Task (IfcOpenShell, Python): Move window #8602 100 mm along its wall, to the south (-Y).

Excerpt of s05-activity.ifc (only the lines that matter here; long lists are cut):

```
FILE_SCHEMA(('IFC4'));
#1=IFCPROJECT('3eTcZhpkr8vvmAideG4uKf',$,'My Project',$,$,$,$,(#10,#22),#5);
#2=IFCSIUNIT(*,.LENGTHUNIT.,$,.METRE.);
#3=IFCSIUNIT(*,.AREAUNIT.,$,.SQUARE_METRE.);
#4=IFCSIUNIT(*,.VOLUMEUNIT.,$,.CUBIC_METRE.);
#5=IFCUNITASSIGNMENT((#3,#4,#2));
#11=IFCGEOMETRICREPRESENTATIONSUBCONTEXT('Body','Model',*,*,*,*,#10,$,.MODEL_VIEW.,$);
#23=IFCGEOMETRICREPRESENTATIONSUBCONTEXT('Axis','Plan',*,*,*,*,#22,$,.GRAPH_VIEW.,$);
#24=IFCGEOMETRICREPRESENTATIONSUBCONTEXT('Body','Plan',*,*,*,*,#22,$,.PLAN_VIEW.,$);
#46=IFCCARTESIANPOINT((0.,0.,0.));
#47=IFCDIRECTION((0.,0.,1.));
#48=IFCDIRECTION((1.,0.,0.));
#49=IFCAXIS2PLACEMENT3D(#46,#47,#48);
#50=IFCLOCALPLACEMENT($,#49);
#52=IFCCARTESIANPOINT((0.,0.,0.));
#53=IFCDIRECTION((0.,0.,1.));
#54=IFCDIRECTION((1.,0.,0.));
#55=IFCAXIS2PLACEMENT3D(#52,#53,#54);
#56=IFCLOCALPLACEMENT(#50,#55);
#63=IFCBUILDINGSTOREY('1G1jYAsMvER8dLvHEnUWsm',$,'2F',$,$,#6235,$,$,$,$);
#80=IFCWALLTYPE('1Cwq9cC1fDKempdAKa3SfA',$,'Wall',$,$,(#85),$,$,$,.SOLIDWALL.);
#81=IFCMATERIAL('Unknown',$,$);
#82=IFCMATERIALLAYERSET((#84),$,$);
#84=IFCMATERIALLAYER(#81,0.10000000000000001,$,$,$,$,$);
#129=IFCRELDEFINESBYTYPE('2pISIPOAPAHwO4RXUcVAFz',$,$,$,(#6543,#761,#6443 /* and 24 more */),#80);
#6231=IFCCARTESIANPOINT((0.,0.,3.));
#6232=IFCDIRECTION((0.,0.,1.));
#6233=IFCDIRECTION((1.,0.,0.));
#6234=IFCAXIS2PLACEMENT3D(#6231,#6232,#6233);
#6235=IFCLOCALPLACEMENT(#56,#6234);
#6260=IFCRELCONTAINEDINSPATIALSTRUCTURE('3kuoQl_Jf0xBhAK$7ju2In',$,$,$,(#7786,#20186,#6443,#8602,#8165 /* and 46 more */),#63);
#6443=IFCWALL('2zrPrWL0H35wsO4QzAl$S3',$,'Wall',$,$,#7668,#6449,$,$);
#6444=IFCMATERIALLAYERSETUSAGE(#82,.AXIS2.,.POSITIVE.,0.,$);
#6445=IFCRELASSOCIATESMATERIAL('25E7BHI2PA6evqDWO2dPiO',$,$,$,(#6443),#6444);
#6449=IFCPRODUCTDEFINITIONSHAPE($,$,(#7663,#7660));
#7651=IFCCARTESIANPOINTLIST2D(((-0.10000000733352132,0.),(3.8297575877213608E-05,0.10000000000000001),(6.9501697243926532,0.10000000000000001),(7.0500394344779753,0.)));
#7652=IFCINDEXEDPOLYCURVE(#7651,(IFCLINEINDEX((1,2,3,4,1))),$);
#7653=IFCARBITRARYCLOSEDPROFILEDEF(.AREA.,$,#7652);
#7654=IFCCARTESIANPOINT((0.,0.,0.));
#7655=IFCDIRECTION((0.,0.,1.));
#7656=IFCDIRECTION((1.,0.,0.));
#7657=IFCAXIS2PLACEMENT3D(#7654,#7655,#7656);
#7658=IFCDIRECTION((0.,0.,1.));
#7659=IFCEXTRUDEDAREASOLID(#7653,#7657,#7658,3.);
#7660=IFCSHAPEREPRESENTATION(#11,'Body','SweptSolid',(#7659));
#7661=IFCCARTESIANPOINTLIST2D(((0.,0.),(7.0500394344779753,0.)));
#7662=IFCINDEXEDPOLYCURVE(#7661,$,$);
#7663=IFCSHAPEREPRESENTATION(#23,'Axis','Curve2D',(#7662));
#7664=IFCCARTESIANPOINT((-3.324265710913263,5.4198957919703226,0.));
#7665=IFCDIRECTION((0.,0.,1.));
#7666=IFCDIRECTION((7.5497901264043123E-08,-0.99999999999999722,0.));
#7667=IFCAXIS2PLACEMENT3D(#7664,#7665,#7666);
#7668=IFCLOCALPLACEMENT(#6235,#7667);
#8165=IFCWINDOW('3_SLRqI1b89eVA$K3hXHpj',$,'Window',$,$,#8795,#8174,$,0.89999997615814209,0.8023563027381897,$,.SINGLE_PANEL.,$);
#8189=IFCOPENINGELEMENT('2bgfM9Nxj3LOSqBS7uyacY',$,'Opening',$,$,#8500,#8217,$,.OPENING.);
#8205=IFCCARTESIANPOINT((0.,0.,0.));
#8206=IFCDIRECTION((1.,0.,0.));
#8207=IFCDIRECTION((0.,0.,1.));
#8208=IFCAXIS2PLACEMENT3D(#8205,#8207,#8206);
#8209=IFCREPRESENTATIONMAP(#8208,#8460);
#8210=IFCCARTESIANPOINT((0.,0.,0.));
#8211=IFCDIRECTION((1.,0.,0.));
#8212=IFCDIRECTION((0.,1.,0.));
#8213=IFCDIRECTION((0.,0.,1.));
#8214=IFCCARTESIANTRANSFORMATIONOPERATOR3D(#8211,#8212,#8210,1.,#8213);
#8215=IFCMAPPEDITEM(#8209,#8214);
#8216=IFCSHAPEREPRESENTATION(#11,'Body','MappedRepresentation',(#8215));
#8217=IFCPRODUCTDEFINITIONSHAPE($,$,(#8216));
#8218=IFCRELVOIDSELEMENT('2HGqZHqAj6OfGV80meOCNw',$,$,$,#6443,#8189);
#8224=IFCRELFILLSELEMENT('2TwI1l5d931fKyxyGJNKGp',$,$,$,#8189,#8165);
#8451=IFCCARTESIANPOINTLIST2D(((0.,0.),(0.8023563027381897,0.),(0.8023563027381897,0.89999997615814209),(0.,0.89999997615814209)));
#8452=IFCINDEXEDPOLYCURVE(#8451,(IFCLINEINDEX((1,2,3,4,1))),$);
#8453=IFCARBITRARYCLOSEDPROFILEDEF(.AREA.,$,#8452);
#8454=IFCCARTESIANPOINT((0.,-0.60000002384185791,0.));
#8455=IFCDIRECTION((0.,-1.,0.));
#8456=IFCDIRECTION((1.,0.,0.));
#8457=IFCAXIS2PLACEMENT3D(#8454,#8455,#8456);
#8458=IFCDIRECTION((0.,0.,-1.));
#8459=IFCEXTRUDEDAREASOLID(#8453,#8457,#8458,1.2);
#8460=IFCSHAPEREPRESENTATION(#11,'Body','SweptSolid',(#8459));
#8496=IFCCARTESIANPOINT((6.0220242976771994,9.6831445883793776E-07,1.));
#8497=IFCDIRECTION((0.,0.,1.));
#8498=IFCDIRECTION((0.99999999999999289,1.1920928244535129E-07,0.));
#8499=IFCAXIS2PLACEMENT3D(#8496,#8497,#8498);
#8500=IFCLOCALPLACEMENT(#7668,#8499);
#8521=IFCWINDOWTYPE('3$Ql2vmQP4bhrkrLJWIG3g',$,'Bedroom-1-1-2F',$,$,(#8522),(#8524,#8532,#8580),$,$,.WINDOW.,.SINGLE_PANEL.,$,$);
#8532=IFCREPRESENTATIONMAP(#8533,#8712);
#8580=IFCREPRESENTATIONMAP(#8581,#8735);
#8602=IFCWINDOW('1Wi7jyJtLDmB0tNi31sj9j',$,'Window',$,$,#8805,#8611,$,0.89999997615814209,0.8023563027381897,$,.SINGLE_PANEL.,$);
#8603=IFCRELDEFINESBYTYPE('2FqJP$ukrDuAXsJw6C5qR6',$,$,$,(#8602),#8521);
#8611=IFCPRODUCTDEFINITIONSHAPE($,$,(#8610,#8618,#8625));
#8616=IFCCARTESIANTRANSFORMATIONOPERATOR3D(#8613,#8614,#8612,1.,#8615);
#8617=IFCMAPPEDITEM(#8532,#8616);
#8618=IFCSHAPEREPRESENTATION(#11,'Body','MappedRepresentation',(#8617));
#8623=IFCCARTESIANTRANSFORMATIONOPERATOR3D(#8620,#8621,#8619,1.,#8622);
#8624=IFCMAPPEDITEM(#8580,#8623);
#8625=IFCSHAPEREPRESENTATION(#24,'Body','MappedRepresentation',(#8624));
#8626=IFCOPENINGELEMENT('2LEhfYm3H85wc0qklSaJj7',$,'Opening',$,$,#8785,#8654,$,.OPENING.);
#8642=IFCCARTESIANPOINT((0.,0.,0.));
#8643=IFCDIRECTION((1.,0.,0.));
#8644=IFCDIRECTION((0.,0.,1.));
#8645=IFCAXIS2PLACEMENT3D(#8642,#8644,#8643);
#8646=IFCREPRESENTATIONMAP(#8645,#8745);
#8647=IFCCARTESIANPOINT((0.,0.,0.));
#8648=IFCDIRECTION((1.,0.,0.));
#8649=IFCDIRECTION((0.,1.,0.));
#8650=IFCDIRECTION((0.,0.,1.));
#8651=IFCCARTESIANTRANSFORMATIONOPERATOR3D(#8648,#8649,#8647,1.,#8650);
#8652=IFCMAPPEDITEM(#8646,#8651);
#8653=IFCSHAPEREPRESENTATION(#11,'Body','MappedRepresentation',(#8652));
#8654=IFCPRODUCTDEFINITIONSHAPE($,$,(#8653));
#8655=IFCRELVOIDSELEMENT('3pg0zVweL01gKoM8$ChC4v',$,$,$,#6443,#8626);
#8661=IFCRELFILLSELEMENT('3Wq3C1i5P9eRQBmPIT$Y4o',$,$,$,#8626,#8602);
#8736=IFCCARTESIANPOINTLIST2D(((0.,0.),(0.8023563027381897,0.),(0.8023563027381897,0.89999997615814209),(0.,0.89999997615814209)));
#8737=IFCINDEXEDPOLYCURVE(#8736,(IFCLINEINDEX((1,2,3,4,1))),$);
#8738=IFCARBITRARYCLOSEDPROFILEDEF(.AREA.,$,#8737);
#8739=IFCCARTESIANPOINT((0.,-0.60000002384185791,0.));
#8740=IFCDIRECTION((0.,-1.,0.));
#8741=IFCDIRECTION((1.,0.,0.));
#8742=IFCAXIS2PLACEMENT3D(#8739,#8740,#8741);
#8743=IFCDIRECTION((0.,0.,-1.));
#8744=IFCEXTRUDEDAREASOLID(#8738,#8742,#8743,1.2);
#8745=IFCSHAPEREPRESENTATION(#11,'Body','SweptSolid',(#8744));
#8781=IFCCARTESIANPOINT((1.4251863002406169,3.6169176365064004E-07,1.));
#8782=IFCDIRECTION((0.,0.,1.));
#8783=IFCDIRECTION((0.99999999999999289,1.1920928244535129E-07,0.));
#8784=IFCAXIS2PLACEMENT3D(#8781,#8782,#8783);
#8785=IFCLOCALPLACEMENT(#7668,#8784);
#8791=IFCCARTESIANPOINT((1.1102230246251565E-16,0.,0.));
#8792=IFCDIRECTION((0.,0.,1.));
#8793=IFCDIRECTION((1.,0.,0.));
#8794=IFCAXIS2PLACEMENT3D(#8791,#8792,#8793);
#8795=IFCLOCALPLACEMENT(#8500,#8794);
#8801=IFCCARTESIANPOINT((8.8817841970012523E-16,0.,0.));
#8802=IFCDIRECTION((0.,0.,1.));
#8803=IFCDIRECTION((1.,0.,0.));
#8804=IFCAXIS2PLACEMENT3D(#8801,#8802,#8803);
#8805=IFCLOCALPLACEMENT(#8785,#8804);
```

```python
import ifcopenshell
import ifcopenshell.api.geometry
import ifcopenshell.util.placement
import ifcopenshell.util.unit

model = ifcopenshell.open("s05-activity.ifc")
unit_scale = ifcopenshell.util.unit.calculate_unit_scale(model)

window = model.by_id(8602)
opening = window.FillsVoids[0].RelatingOpeningElement
wall = opening.VoidsElements[0].RelatingBuildingElement

wall_matrix = ifcopenshell.util.placement.get_local_placement(wall.ObjectPlacement)
shift = wall_matrix[:3, 0] * 0.1 / unit_scale
before = ifcopenshell.util.placement.get_local_placement(window.ObjectPlacement)[:3, 3].copy()

# The window is placed relative to its opening, so it follows when the opening moves.
matrix = ifcopenshell.util.placement.get_local_placement(opening.ObjectPlacement)
matrix[:3, 3] += shift
ifcopenshell.api.geometry.edit_object_placement(
    model, product=opening, matrix=matrix, is_si=False, should_transform_children=True
)

after = ifcopenshell.util.placement.get_local_placement(window.ObjectPlacement)[:3, 3]
print("window moved by", (after - before).round(3) + 0.0)

model.write("s05-activity_rev.ifc")
```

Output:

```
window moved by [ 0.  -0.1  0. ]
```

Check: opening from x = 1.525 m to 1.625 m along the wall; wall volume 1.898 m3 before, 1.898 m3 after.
